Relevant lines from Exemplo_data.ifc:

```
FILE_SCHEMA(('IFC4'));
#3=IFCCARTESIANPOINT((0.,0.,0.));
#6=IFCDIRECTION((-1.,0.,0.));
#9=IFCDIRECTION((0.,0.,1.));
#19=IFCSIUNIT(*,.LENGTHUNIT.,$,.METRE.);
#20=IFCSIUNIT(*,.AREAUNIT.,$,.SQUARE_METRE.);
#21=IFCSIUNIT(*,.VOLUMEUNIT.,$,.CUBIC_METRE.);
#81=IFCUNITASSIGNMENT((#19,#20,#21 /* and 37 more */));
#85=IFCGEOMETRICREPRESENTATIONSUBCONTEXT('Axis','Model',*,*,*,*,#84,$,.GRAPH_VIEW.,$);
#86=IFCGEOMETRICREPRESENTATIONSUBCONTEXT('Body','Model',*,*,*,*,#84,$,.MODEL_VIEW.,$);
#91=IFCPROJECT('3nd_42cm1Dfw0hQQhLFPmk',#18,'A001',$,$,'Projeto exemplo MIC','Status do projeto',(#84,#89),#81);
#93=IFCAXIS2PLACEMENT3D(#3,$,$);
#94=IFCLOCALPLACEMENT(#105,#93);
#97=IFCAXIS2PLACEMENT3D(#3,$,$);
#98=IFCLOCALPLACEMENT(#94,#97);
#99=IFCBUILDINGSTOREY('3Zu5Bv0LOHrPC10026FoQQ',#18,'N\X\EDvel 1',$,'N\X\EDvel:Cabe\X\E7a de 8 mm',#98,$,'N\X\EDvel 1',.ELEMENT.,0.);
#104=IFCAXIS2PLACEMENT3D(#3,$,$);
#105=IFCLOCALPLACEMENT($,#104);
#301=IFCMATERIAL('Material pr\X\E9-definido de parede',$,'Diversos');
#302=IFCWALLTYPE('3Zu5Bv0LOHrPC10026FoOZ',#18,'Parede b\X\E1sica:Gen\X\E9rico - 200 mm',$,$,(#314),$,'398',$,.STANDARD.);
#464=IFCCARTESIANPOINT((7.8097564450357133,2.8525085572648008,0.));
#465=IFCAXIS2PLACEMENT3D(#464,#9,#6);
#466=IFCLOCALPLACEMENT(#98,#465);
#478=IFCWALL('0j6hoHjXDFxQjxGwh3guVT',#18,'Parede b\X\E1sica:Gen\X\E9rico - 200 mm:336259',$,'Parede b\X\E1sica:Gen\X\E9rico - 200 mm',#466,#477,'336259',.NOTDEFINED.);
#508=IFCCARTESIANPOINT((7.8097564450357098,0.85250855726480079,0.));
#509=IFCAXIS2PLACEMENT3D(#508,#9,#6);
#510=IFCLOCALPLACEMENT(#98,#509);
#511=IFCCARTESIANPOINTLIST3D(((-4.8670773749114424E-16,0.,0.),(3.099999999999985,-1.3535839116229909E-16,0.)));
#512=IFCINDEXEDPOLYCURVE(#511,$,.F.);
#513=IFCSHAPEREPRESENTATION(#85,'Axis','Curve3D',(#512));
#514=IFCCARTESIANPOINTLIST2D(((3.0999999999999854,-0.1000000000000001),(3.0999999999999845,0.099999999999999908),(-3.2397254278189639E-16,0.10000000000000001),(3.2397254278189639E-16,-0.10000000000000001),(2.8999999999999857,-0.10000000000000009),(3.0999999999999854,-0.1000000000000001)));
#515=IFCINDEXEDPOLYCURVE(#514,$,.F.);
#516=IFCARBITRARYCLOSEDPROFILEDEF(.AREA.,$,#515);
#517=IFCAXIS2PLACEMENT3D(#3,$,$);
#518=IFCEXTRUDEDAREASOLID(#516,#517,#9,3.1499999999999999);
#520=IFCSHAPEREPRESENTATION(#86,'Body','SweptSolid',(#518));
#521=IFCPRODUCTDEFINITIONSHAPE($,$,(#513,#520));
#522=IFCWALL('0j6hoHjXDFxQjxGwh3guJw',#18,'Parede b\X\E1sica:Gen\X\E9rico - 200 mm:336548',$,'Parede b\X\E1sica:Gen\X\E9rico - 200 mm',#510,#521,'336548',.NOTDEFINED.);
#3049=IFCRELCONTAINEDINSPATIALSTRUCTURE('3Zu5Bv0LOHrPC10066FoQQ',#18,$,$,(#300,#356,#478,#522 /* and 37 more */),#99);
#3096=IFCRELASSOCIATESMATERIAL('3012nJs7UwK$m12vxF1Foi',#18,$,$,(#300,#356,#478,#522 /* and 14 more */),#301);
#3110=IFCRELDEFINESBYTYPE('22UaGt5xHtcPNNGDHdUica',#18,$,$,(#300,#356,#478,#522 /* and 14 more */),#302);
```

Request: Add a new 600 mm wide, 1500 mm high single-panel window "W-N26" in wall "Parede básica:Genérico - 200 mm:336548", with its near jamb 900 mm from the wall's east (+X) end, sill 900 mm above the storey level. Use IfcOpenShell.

```python
import numpy as np
import ifcopenshell
import ifcopenshell.api.feature
import ifcopenshell.api.geometry
import ifcopenshell.api.root
import ifcopenshell.api.spatial
import ifcopenshell.geom
import ifcopenshell.util.element
import ifcopenshell.util.placement
import ifcopenshell.util.representation
import ifcopenshell.util.shape
import ifcopenshell.util.unit

model = ifcopenshell.open("Exemplo_data.ifc")
unit_scale = ifcopenshell.util.unit.calculate_unit_scale(model)
settings = ifcopenshell.geom.settings()


def volume(element):
    """Net volume in cubic metres, openings subtracted."""
    shape = ifcopenshell.geom.create_shape(settings, element)
    return ifcopenshell.util.shape.get_volume(shape.geometry)


wall = model.by_guid("0j6hoHjXDFxQjxGwh3guJw")
storey = ifcopenshell.util.element.get_container(wall, ifc_class="IfcBuildingStorey")
context = ifcopenshell.util.representation.get_context(model, "Model", "Body", "MODEL_VIEW")
before = volume(wall)

width, height, from_end, sill = 0.6, 1.5, 0.9, 0.9  # metres

# The wall runs along its own X axis, and the end named is its -X end.
wall_shape = ifcopenshell.geom.create_shape(settings, wall)
x, y, z = ifcopenshell.util.shape.get_vertices(wall_shape.geometry).T
start = x.min() + from_end
face, thickness = float(y.min()), float(y.max() - y.min())
wall_matrix = ifcopenshell.util.placement.get_local_placement(wall.ObjectPlacement)
level = ifcopenshell.util.placement.get_local_placement(storey.ObjectPlacement)[2, 3]


def in_wall(x, y):
    """Placement at x, y metres in the wall's axes, at sill height."""
    matrix = wall_matrix.copy()
    matrix[:, 3] = wall_matrix @ np.array([x / unit_scale, y / unit_scale, 0.0, 1.0])
    matrix[2, 3] = level + sill / unit_scale
    return matrix


# Opening: a box that overshoots both wall faces by 50 mm.
opening = ifcopenshell.api.root.create_entity(model, ifc_class="IfcOpeningElement", predefined_type="OPENING")
box = ifcopenshell.api.geometry.add_wall_representation(
    model, context=context, length=width, height=height, thickness=thickness + 0.1
)
ifcopenshell.api.geometry.assign_representation(model, product=opening, representation=box)
ifcopenshell.api.geometry.edit_object_placement(model, product=opening, matrix=in_wall(start, face - 0.05), is_si=False)
ifcopenshell.api.feature.add_feature(model, feature=opening, element=wall)

window = ifcopenshell.api.root.create_entity(model, ifc_class="IfcWindow", name="W-N26", predefined_type="WINDOW")
window.OverallWidth, window.OverallHeight = width / unit_scale, height / unit_scale
window.PartitioningType = "SINGLE_PANEL"
body = ifcopenshell.api.geometry.add_window_representation(
    model,
    context=context,
    overall_width=window.OverallWidth,
    overall_height=window.OverallHeight,
    partition_type="SINGLE_PANEL",
)
ifcopenshell.api.geometry.assign_representation(model, product=window, representation=body)
ifcopenshell.api.spatial.assign_container(model, products=[window], relating_structure=storey)
ifcopenshell.api.feature.add_filling(model, opening=opening, element=window)

# Centre the window in the wall's thickness.
ifcopenshell.api.geometry.edit_object_placement(model, product=window, matrix=in_wall(start, face), is_si=False)
window_shape = ifcopenshell.geom.create_shape(settings, window)
depth = ifcopenshell.util.shape.get_vertices(window_shape.geometry)[:, 1]
offset = face + thickness / 2 - (depth.min() + depth.max()) / 2
ifcopenshell.api.geometry.edit_object_placement(model, product=window, matrix=in_wall(start, offset), is_si=False)

after = volume(wall)

print(f"wall volume {before:.3f} -> {after:.3f} m3")

model.write("Exemplo_data_updated.ifc")
```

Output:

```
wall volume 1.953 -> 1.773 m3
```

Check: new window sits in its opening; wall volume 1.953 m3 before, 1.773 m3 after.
